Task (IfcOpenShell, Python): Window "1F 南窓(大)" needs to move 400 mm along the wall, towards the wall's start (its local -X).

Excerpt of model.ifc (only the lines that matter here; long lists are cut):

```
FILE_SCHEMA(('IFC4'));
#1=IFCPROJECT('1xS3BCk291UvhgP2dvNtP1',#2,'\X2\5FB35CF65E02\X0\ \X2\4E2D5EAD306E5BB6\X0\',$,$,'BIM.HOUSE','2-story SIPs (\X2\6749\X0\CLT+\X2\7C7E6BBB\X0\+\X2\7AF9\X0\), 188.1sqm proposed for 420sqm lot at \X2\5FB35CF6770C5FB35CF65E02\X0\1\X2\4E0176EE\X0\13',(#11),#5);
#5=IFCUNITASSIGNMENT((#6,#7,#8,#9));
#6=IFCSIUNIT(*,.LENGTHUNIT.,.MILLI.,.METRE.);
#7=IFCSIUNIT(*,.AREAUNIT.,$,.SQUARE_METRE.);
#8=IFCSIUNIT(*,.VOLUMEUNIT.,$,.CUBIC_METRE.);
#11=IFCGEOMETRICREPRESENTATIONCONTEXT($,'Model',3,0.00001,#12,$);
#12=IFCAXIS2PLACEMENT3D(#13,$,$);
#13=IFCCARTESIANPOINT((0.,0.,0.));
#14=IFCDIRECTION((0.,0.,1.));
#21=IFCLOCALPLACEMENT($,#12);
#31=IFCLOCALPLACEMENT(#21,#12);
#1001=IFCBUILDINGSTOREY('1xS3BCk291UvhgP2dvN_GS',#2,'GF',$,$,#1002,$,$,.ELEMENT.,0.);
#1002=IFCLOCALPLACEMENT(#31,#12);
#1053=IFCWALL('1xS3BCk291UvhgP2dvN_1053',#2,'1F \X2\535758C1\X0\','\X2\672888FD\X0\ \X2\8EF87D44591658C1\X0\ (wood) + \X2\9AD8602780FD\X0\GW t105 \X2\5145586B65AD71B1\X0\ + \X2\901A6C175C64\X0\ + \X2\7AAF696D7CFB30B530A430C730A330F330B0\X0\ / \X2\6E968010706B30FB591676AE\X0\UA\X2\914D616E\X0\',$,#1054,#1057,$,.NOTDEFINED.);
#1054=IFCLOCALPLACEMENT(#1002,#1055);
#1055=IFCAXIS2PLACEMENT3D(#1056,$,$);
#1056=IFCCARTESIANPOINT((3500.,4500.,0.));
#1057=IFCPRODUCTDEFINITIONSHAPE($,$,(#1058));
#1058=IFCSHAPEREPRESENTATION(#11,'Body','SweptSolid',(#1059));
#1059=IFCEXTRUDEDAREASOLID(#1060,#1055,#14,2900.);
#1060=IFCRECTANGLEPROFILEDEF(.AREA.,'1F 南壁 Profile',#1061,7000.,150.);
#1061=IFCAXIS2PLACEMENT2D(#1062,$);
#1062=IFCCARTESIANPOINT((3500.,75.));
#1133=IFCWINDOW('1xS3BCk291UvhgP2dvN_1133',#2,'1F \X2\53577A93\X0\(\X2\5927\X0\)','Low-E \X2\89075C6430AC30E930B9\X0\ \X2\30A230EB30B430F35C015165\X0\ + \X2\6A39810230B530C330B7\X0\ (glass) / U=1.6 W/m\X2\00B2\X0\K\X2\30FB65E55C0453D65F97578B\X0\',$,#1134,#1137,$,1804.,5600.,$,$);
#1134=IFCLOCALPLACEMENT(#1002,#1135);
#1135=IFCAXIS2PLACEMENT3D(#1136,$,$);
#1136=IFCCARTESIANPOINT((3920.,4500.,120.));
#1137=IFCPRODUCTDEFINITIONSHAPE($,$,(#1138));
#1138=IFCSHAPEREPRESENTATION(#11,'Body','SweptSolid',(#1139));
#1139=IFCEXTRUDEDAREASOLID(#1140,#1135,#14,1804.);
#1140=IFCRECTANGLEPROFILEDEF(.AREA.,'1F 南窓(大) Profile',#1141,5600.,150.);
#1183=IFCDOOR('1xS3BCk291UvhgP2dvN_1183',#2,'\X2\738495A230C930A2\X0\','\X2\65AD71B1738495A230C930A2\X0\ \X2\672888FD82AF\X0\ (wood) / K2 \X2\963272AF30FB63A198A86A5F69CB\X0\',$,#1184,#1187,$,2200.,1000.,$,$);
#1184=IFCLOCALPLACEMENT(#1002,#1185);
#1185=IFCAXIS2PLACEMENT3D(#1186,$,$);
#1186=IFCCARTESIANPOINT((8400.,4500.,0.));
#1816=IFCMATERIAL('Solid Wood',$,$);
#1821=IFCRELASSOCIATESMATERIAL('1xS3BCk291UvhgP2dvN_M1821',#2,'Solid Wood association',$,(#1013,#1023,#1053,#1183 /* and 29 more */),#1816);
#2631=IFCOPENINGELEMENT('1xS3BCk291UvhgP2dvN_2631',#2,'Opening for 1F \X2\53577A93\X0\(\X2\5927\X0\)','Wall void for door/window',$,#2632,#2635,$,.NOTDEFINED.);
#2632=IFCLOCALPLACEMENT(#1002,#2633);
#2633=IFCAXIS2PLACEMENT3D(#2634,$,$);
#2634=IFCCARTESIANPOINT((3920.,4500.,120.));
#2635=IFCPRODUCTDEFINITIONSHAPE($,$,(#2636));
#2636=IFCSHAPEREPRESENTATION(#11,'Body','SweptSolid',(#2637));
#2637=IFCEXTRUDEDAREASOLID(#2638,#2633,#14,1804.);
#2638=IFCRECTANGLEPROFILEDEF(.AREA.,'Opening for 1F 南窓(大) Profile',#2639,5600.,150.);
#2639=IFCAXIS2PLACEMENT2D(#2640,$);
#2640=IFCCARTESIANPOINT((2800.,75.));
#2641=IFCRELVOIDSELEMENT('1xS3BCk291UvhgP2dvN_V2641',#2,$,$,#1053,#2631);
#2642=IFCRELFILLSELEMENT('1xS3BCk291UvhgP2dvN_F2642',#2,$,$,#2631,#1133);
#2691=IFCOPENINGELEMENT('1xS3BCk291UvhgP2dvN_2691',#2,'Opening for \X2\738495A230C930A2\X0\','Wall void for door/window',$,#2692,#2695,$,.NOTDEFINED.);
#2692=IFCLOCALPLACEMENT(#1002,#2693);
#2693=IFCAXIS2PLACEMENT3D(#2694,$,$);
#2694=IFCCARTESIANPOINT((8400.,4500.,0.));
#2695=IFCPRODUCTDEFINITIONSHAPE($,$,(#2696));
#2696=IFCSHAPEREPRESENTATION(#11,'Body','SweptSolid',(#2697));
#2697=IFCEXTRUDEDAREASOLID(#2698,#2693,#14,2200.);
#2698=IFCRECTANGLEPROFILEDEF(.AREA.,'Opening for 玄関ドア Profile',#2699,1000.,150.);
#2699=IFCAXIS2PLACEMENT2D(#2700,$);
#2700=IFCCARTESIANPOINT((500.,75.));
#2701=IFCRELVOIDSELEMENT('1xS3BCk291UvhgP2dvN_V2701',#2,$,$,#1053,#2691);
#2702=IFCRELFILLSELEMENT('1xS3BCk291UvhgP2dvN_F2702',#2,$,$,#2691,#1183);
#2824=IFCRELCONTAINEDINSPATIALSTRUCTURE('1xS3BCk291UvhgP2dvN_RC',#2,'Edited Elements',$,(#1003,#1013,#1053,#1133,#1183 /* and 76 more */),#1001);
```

```python
import ifcopenshell
import ifcopenshell.api.geometry
import ifcopenshell.util.placement

model = ifcopenshell.open("model.ifc")

window = model.by_guid("1xS3BCk291UvhgP2dvN_1133")
opening = window.FillsVoids[0].RelatingOpeningElement
wall = opening.VoidsElements[0].RelatingBuildingElement

wall_matrix = ifcopenshell.util.placement.get_local_placement(wall.ObjectPlacement)
shift = wall_matrix[:3, 0] * -400.0
before = ifcopenshell.util.placement.get_local_placement(window.ObjectPlacement)[:3, 3].copy()

# The window is not placed relative to its opening, so move both.
for product in (opening, window):
    matrix = ifcopenshell.util.placement.get_local_placement(product.ObjectPlacement)
    matrix[:3, 3] += shift
    ifcopenshell.api.geometry.edit_object_placement(model, product=product, matrix=matrix, is_si=False)

after = ifcopenshell.util.placement.get_local_placement(window.ObjectPlacement)[:3, 3]
print("window moved by", (after - before).round(3) + 0.0)

model.write("model_rev.ifc")
```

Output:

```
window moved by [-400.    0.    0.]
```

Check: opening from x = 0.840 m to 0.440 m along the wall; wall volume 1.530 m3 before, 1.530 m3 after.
